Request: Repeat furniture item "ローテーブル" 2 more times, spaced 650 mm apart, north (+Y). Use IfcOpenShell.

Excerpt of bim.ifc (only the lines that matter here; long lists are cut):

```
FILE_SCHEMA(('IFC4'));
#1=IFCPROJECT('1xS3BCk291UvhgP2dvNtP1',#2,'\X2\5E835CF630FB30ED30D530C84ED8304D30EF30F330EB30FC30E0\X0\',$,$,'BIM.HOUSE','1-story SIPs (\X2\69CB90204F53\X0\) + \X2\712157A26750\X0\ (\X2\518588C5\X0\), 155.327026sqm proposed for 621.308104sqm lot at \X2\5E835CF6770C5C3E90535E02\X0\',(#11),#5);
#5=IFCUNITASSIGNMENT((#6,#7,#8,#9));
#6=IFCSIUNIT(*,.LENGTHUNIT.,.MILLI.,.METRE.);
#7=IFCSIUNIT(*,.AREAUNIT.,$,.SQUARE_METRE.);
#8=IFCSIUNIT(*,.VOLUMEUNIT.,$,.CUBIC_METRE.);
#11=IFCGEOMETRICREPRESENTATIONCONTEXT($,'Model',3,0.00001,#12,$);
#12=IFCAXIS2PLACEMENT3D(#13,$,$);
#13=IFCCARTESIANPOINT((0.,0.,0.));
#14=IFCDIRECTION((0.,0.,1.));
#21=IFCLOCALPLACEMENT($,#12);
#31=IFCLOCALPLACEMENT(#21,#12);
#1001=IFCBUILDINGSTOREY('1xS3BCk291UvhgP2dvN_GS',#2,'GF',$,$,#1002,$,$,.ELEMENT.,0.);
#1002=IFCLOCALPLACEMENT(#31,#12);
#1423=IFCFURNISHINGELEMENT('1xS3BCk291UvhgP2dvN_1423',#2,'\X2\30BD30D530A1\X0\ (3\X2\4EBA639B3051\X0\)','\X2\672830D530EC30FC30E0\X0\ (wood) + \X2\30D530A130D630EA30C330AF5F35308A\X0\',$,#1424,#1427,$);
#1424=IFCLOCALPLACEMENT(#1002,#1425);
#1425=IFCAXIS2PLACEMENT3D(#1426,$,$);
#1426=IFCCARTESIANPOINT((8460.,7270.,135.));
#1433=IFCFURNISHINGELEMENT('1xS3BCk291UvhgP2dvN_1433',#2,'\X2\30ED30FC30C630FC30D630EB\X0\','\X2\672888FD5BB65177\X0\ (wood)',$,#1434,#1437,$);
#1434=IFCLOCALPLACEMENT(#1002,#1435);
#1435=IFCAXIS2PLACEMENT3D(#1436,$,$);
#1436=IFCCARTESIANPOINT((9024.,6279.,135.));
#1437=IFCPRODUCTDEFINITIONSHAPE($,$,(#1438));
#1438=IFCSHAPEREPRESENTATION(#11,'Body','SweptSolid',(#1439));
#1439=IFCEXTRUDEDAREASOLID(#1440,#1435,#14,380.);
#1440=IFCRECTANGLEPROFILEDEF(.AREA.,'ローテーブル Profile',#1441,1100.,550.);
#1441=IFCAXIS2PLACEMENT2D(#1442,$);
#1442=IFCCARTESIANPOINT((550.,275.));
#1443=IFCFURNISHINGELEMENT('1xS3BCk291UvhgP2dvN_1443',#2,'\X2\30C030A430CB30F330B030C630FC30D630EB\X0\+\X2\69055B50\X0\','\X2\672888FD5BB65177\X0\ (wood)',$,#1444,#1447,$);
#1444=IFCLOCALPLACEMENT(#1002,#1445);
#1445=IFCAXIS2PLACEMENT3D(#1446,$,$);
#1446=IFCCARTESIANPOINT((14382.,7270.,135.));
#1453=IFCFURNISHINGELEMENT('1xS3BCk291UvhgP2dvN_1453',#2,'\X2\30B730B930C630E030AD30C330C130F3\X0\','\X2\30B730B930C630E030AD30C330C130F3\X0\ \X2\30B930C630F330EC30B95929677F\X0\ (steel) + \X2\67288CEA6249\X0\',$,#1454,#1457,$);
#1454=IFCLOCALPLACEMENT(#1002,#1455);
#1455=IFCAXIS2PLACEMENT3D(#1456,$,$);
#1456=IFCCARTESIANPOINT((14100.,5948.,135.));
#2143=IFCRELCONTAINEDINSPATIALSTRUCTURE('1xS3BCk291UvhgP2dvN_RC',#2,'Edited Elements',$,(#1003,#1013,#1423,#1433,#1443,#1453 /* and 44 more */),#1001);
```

```python
import numpy as np
import ifcopenshell
import ifcopenshell.api.geometry
import ifcopenshell.api.root
import ifcopenshell.util.element
import ifcopenshell.util.placement

model = ifcopenshell.open("bim.ifc")


def reuse_history(source, copy):
    """copy_class also copies each property set's owner history, people and application; keep the originals."""
    for rel in copy.IsDefinedBy:
        if rel.is_a("IfcRelDefinesByProperties") and (history := rel.RelatingPropertyDefinition.OwnerHistory):
            rel.RelatingPropertyDefinition.OwnerHistory = source.OwnerHistory
            ifcopenshell.util.element.remove_deep2(model, history)


source = model.by_guid("1xS3BCk291UvhgP2dvN_1433")
base = ifcopenshell.util.placement.get_local_placement(source.ObjectPlacement)
step = np.array([0.0, 1.0, 0.0]) * 650.0

for i in range(1, 3):
    copy = ifcopenshell.api.root.copy_class(model, product=source)
    copy.Representation = ifcopenshell.util.element.copy_deep(
        model, source.Representation, exclude=["IfcGeometricRepresentationContext", "IfcRepresentationMap"]
    )
    reuse_history(source, copy)
    matrix = base.copy()
    matrix[:3, 3] += i * step
    print("added at", matrix[:3, 3].round(3) + 0.0)
    ifcopenshell.api.geometry.edit_object_placement(model, product=copy, matrix=matrix, is_si=False)

model.write("bim_updated.ifc")
```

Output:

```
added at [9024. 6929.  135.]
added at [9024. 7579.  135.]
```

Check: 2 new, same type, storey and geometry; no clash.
